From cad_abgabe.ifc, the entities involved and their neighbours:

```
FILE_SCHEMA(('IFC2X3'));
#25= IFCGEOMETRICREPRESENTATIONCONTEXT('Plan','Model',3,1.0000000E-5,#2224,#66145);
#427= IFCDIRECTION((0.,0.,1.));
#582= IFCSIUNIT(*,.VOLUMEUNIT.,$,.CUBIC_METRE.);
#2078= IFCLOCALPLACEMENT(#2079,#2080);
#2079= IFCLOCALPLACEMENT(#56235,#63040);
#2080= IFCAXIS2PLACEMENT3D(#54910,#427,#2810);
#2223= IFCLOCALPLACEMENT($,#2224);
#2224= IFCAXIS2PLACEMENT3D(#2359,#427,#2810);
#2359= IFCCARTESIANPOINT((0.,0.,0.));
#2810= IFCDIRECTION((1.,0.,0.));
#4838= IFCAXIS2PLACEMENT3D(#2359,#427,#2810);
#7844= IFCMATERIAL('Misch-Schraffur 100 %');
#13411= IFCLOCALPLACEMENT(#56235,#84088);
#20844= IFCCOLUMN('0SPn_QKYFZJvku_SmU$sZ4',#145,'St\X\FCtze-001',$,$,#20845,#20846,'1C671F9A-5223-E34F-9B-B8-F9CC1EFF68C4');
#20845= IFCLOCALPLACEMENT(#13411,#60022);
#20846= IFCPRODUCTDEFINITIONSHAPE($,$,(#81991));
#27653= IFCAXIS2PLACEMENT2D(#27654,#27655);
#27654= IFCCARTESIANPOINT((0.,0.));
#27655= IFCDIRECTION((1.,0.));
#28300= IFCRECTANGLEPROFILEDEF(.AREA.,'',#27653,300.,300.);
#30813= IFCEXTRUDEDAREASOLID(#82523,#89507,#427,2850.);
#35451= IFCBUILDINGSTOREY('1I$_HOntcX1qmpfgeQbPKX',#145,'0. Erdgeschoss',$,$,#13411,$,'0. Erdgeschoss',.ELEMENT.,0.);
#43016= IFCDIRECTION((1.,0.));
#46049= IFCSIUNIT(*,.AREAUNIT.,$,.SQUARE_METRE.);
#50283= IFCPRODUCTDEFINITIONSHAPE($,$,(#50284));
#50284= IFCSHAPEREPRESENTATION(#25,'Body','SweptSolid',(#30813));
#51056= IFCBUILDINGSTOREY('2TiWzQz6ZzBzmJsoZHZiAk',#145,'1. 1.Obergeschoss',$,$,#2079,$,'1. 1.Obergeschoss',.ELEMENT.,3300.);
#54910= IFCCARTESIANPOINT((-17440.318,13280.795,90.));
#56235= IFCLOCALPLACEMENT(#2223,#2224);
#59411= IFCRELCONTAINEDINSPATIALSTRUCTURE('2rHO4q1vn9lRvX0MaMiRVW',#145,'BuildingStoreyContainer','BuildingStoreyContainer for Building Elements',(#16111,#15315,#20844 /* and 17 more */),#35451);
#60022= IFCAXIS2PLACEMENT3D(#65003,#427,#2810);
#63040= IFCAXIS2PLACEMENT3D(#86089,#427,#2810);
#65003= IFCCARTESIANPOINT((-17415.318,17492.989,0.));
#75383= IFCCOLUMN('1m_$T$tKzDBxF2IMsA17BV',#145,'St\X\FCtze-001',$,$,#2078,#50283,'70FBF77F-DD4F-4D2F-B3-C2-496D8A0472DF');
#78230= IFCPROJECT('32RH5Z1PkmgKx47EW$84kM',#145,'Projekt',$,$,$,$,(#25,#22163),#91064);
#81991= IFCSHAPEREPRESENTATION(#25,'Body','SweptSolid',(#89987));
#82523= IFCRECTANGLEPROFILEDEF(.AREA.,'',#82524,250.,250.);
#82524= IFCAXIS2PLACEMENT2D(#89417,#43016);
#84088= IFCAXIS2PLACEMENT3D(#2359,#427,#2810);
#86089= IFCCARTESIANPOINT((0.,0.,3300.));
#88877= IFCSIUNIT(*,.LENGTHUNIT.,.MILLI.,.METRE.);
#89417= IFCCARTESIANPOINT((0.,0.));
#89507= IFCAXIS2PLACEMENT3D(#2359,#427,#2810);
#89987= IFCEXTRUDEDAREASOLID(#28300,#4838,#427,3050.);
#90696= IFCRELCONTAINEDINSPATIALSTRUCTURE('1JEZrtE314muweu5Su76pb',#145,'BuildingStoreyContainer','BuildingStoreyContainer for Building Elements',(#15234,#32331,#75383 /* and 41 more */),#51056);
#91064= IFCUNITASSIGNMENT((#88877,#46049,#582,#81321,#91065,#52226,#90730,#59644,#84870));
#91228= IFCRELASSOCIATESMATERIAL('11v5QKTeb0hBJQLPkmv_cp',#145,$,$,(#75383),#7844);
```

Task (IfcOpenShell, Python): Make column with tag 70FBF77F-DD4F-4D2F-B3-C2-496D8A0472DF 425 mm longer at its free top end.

```python
import ifcopenshell

model = ifcopenshell.open("cad_abgabe.ifc")

member = model.by_id(75383)
change = 425.0

# The extrusion runs towards the end named, so only its depth changes.
body = next(r for r in member.Representation.Representations if r.RepresentationIdentifier == "Body")
solid = body.Items[0]
old_length = solid.Depth
solid.Depth += change

print(f"length {old_length:g} -> {solid.Depth:g}")

model.write("cad_abgabe_v2.ifc")
```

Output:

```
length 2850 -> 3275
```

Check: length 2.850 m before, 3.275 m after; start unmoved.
